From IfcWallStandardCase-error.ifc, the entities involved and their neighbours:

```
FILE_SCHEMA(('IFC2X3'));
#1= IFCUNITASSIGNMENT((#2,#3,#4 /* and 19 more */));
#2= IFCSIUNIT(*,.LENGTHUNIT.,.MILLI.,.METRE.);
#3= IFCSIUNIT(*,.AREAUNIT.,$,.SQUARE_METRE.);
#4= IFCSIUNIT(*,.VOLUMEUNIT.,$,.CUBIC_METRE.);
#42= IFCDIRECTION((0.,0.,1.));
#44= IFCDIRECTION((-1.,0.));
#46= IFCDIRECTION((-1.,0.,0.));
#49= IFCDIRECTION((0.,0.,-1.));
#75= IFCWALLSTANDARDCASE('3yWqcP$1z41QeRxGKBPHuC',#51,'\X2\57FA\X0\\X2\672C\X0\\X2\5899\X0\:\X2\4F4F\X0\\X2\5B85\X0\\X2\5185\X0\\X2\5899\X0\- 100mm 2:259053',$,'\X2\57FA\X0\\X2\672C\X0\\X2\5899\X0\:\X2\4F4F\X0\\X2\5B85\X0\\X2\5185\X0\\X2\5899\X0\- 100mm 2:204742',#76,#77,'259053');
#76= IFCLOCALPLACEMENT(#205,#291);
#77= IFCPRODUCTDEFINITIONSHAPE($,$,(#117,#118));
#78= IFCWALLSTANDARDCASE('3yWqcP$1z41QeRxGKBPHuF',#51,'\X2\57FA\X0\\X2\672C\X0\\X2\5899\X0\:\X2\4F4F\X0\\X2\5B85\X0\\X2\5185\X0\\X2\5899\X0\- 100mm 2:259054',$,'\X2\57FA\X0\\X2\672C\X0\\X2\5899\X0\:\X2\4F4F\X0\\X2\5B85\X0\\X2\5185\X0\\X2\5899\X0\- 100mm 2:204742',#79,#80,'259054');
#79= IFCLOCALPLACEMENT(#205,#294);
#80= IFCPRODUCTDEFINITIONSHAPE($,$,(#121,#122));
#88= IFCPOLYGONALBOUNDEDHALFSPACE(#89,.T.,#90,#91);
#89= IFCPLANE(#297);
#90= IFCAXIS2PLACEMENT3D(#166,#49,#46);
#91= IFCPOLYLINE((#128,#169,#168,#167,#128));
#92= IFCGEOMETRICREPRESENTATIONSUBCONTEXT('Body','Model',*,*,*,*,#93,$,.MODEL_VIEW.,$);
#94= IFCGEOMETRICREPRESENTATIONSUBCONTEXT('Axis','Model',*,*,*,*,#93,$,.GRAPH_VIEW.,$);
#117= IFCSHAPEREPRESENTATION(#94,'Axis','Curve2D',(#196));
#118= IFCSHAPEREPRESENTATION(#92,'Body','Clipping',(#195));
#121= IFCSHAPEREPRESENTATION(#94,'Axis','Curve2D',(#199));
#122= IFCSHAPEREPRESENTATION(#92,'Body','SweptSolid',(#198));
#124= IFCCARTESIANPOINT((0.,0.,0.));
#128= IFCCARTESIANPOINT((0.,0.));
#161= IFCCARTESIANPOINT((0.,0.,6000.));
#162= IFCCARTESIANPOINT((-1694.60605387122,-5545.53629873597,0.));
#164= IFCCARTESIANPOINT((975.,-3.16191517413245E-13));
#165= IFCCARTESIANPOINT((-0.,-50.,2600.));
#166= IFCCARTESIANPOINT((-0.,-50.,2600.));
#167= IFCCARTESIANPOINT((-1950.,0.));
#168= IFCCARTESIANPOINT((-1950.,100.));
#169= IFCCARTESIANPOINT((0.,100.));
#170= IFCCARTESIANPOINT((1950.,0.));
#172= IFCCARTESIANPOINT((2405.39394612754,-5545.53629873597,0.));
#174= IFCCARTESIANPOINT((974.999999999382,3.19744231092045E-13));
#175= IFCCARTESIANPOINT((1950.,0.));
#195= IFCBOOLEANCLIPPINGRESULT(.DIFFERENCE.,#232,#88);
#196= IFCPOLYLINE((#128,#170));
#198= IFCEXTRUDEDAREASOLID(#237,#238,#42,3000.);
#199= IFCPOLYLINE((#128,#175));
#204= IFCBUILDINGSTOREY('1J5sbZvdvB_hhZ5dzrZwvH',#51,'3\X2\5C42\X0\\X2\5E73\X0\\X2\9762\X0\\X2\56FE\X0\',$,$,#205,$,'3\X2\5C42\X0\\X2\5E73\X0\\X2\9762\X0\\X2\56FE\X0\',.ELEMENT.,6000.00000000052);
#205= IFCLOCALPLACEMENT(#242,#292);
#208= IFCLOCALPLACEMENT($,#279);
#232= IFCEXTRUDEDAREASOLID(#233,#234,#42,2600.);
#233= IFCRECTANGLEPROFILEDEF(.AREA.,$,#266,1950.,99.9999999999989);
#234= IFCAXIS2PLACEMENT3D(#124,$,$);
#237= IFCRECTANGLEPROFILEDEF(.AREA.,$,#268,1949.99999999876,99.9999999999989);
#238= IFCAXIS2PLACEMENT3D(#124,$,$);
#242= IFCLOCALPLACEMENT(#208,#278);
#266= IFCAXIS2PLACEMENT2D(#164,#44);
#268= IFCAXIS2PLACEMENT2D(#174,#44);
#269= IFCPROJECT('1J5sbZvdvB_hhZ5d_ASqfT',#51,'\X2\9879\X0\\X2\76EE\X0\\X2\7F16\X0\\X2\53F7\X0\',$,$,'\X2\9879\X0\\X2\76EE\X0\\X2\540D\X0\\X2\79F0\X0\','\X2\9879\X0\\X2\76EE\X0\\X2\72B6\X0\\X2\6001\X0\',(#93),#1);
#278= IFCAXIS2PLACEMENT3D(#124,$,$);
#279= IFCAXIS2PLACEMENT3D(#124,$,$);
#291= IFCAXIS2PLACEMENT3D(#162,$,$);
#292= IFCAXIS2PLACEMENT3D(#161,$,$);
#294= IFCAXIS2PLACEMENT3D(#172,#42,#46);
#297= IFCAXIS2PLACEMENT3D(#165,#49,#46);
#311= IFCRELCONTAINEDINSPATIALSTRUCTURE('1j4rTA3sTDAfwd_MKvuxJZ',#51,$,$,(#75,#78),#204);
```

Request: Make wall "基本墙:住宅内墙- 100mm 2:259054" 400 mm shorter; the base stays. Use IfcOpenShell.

```python
import ifcopenshell
import ifcopenshell.geom
import ifcopenshell.util.representation
import ifcopenshell.util.shape

model = ifcopenshell.open("IfcWallStandardCase-error.ifc")
settings = ifcopenshell.geom.settings()


def volume(element):
    """Net volume in cubic metres, openings subtracted."""
    shape = ifcopenshell.geom.create_shape(settings, element)
    return ifcopenshell.util.shape.get_volume(shape.geometry)


wall = model.by_id(78)
before = volume(wall)

body = ifcopenshell.util.representation.get_representation(wall, "Model", "Body")
solid = body.Items[0]
old_height = solid.Depth
solid.Depth -= 400.0
after = volume(wall)

print(f"height {old_height:g} -> {solid.Depth:g}, volume {before:.3f} -> {after:.3f} m3")

model.write("IfcWallStandardCase-error_v2.ifc")
```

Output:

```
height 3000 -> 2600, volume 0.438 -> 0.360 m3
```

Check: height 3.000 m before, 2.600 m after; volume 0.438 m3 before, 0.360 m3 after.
